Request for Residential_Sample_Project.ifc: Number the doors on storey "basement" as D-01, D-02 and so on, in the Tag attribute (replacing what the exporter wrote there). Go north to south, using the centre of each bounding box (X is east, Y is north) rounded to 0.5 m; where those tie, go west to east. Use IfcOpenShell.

First a look at what the model holds.

```python
import ifcopenshell
import ifcopenshell.util.element
import ifcopenshell.util.placement

model = ifcopenshell.open("Residential_Sample_Project.ifc")
print(model.schema)
storey = next(s for s in model.by_type("IfcBuildingStorey") if s.Name == "basement")
doors = [e for e in ifcopenshell.util.element.get_decomposition(storey) if e.is_a("IfcDoor")]
for e in sorted(doors, key=lambda e: e.id()):
    origin = ifcopenshell.util.placement.get_local_placement(e.ObjectPlacement)[:3, 3]
    print(e.id(), e.Tag, e.Name, origin.round(2) + 0.0, sep=" | ")
```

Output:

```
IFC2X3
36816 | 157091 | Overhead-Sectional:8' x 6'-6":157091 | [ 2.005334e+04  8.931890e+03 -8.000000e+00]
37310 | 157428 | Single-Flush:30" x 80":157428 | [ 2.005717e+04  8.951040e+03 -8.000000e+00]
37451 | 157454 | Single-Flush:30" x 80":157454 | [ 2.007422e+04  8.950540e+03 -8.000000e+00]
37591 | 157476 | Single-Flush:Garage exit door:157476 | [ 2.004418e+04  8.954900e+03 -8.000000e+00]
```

```python
import ifcopenshell
import ifcopenshell.geom
import ifcopenshell.util.element
import ifcopenshell.util.shape

model = ifcopenshell.open("Residential_Sample_Project.ifc")
settings = ifcopenshell.geom.settings()
settings.set("use-world-coords", True)


def centre(element):
    shape = ifcopenshell.geom.create_shape(settings, element)
    return ifcopenshell.util.shape.get_bbox_centroid(shape.geometry)


storey = next(s for s in model.by_type("IfcBuildingStorey") if s.Name == "basement")
doors = [e for e in ifcopenshell.util.element.get_decomposition(storey) if e.is_a("IfcDoor")]

# Insertion points can sit at a corner or the storey origin, so sort by the geometry (in metres).
centres = {e: centre(e) for e in doors}
doors.sort(key=lambda e: (-round(centres[e][1] / 0.5), centres[e][0]))

for i, e in enumerate(doors, start=1):
    number = f"D-{i:02d}"
    e.Tag = number
    print(e.id(), number)

model.write("Residential_Sample_Project_edited.ifc")
```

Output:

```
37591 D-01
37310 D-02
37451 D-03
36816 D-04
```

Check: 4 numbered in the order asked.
